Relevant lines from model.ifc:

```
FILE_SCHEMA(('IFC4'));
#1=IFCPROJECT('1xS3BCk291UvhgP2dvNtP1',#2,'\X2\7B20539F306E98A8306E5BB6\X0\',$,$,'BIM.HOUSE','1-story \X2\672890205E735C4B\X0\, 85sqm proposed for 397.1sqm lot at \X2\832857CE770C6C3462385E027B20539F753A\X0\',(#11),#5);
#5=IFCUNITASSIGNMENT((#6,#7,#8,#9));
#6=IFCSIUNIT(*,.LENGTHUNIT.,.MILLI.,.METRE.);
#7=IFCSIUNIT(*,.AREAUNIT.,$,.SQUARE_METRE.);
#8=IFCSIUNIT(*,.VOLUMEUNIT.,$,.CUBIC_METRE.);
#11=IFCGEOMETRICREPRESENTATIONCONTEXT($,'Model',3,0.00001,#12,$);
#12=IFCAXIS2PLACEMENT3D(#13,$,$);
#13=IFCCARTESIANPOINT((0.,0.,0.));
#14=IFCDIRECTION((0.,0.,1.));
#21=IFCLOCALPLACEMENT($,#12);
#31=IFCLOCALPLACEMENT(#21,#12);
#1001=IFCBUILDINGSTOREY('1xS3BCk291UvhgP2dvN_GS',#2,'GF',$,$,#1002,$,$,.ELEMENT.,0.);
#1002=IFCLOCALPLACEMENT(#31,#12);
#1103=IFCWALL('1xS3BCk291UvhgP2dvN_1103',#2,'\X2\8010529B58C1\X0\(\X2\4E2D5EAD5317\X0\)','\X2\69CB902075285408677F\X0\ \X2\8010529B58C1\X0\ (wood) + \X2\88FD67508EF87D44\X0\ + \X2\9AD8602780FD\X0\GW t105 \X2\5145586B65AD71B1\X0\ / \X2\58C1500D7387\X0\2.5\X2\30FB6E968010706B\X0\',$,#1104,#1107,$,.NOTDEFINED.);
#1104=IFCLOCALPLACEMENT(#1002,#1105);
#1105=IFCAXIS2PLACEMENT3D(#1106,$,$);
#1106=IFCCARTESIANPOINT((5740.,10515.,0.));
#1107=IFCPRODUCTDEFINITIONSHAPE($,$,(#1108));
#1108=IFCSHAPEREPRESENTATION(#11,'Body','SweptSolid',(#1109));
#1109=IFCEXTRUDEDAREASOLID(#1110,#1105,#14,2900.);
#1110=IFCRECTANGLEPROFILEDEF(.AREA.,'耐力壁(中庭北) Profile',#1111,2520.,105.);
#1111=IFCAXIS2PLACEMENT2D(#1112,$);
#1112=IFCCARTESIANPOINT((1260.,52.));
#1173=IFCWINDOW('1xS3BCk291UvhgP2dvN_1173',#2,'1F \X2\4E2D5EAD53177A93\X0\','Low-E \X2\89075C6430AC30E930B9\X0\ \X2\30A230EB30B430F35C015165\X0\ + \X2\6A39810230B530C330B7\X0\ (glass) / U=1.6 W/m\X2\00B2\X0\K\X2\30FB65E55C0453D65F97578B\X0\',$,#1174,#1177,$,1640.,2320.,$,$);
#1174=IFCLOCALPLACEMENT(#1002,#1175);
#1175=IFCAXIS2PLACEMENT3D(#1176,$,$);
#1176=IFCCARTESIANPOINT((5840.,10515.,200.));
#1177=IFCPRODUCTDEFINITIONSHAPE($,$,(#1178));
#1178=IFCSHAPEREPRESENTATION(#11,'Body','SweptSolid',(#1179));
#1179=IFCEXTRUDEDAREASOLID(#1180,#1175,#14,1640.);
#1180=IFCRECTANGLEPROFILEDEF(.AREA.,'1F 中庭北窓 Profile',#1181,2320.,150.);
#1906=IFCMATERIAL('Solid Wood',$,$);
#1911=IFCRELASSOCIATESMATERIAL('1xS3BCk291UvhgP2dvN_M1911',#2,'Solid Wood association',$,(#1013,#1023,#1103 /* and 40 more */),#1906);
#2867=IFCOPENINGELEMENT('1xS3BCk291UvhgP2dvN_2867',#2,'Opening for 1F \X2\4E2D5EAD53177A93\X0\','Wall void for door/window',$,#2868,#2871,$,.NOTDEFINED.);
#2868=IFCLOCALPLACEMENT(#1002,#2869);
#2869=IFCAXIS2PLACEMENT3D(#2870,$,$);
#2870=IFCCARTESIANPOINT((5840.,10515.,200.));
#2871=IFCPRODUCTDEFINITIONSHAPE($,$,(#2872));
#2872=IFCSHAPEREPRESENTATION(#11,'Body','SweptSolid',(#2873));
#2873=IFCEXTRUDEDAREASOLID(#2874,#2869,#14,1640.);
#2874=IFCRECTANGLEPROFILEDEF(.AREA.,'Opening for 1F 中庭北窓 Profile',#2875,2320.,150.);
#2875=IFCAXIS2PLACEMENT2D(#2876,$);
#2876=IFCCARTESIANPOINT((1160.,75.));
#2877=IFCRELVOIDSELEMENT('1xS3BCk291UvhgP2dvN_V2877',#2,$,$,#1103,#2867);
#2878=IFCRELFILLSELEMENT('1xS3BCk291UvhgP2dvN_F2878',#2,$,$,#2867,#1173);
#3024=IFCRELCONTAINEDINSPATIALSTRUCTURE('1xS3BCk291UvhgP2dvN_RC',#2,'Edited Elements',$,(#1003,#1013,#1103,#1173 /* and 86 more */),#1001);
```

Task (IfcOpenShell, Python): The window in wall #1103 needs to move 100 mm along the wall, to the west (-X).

```python
import ifcopenshell
import ifcopenshell.api.geometry
import ifcopenshell.util.placement

model = ifcopenshell.open("model.ifc")

window = model.by_id(1173)
opening = window.FillsVoids[0].RelatingOpeningElement
wall = opening.VoidsElements[0].RelatingBuildingElement

wall_matrix = ifcopenshell.util.placement.get_local_placement(wall.ObjectPlacement)
shift = wall_matrix[:3, 0] * -100.0
before = ifcopenshell.util.placement.get_local_placement(window.ObjectPlacement)[:3, 3].copy()

# The window is not placed relative to its opening, so move both.
for product in (opening, window):
    matrix = ifcopenshell.util.placement.get_local_placement(product.ObjectPlacement)
    matrix[:3, 3] += shift
    ifcopenshell.api.geometry.edit_object_placement(model, product=product, matrix=matrix, is_si=False)

after = ifcopenshell.util.placement.get_local_placement(window.ObjectPlacement)[:3, 3]
print("window moved by", (after - before).round(3) + 0.0)

model.write("model_rev.ifc")
```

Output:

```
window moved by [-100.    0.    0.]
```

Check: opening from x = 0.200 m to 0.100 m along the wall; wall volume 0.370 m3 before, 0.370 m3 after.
